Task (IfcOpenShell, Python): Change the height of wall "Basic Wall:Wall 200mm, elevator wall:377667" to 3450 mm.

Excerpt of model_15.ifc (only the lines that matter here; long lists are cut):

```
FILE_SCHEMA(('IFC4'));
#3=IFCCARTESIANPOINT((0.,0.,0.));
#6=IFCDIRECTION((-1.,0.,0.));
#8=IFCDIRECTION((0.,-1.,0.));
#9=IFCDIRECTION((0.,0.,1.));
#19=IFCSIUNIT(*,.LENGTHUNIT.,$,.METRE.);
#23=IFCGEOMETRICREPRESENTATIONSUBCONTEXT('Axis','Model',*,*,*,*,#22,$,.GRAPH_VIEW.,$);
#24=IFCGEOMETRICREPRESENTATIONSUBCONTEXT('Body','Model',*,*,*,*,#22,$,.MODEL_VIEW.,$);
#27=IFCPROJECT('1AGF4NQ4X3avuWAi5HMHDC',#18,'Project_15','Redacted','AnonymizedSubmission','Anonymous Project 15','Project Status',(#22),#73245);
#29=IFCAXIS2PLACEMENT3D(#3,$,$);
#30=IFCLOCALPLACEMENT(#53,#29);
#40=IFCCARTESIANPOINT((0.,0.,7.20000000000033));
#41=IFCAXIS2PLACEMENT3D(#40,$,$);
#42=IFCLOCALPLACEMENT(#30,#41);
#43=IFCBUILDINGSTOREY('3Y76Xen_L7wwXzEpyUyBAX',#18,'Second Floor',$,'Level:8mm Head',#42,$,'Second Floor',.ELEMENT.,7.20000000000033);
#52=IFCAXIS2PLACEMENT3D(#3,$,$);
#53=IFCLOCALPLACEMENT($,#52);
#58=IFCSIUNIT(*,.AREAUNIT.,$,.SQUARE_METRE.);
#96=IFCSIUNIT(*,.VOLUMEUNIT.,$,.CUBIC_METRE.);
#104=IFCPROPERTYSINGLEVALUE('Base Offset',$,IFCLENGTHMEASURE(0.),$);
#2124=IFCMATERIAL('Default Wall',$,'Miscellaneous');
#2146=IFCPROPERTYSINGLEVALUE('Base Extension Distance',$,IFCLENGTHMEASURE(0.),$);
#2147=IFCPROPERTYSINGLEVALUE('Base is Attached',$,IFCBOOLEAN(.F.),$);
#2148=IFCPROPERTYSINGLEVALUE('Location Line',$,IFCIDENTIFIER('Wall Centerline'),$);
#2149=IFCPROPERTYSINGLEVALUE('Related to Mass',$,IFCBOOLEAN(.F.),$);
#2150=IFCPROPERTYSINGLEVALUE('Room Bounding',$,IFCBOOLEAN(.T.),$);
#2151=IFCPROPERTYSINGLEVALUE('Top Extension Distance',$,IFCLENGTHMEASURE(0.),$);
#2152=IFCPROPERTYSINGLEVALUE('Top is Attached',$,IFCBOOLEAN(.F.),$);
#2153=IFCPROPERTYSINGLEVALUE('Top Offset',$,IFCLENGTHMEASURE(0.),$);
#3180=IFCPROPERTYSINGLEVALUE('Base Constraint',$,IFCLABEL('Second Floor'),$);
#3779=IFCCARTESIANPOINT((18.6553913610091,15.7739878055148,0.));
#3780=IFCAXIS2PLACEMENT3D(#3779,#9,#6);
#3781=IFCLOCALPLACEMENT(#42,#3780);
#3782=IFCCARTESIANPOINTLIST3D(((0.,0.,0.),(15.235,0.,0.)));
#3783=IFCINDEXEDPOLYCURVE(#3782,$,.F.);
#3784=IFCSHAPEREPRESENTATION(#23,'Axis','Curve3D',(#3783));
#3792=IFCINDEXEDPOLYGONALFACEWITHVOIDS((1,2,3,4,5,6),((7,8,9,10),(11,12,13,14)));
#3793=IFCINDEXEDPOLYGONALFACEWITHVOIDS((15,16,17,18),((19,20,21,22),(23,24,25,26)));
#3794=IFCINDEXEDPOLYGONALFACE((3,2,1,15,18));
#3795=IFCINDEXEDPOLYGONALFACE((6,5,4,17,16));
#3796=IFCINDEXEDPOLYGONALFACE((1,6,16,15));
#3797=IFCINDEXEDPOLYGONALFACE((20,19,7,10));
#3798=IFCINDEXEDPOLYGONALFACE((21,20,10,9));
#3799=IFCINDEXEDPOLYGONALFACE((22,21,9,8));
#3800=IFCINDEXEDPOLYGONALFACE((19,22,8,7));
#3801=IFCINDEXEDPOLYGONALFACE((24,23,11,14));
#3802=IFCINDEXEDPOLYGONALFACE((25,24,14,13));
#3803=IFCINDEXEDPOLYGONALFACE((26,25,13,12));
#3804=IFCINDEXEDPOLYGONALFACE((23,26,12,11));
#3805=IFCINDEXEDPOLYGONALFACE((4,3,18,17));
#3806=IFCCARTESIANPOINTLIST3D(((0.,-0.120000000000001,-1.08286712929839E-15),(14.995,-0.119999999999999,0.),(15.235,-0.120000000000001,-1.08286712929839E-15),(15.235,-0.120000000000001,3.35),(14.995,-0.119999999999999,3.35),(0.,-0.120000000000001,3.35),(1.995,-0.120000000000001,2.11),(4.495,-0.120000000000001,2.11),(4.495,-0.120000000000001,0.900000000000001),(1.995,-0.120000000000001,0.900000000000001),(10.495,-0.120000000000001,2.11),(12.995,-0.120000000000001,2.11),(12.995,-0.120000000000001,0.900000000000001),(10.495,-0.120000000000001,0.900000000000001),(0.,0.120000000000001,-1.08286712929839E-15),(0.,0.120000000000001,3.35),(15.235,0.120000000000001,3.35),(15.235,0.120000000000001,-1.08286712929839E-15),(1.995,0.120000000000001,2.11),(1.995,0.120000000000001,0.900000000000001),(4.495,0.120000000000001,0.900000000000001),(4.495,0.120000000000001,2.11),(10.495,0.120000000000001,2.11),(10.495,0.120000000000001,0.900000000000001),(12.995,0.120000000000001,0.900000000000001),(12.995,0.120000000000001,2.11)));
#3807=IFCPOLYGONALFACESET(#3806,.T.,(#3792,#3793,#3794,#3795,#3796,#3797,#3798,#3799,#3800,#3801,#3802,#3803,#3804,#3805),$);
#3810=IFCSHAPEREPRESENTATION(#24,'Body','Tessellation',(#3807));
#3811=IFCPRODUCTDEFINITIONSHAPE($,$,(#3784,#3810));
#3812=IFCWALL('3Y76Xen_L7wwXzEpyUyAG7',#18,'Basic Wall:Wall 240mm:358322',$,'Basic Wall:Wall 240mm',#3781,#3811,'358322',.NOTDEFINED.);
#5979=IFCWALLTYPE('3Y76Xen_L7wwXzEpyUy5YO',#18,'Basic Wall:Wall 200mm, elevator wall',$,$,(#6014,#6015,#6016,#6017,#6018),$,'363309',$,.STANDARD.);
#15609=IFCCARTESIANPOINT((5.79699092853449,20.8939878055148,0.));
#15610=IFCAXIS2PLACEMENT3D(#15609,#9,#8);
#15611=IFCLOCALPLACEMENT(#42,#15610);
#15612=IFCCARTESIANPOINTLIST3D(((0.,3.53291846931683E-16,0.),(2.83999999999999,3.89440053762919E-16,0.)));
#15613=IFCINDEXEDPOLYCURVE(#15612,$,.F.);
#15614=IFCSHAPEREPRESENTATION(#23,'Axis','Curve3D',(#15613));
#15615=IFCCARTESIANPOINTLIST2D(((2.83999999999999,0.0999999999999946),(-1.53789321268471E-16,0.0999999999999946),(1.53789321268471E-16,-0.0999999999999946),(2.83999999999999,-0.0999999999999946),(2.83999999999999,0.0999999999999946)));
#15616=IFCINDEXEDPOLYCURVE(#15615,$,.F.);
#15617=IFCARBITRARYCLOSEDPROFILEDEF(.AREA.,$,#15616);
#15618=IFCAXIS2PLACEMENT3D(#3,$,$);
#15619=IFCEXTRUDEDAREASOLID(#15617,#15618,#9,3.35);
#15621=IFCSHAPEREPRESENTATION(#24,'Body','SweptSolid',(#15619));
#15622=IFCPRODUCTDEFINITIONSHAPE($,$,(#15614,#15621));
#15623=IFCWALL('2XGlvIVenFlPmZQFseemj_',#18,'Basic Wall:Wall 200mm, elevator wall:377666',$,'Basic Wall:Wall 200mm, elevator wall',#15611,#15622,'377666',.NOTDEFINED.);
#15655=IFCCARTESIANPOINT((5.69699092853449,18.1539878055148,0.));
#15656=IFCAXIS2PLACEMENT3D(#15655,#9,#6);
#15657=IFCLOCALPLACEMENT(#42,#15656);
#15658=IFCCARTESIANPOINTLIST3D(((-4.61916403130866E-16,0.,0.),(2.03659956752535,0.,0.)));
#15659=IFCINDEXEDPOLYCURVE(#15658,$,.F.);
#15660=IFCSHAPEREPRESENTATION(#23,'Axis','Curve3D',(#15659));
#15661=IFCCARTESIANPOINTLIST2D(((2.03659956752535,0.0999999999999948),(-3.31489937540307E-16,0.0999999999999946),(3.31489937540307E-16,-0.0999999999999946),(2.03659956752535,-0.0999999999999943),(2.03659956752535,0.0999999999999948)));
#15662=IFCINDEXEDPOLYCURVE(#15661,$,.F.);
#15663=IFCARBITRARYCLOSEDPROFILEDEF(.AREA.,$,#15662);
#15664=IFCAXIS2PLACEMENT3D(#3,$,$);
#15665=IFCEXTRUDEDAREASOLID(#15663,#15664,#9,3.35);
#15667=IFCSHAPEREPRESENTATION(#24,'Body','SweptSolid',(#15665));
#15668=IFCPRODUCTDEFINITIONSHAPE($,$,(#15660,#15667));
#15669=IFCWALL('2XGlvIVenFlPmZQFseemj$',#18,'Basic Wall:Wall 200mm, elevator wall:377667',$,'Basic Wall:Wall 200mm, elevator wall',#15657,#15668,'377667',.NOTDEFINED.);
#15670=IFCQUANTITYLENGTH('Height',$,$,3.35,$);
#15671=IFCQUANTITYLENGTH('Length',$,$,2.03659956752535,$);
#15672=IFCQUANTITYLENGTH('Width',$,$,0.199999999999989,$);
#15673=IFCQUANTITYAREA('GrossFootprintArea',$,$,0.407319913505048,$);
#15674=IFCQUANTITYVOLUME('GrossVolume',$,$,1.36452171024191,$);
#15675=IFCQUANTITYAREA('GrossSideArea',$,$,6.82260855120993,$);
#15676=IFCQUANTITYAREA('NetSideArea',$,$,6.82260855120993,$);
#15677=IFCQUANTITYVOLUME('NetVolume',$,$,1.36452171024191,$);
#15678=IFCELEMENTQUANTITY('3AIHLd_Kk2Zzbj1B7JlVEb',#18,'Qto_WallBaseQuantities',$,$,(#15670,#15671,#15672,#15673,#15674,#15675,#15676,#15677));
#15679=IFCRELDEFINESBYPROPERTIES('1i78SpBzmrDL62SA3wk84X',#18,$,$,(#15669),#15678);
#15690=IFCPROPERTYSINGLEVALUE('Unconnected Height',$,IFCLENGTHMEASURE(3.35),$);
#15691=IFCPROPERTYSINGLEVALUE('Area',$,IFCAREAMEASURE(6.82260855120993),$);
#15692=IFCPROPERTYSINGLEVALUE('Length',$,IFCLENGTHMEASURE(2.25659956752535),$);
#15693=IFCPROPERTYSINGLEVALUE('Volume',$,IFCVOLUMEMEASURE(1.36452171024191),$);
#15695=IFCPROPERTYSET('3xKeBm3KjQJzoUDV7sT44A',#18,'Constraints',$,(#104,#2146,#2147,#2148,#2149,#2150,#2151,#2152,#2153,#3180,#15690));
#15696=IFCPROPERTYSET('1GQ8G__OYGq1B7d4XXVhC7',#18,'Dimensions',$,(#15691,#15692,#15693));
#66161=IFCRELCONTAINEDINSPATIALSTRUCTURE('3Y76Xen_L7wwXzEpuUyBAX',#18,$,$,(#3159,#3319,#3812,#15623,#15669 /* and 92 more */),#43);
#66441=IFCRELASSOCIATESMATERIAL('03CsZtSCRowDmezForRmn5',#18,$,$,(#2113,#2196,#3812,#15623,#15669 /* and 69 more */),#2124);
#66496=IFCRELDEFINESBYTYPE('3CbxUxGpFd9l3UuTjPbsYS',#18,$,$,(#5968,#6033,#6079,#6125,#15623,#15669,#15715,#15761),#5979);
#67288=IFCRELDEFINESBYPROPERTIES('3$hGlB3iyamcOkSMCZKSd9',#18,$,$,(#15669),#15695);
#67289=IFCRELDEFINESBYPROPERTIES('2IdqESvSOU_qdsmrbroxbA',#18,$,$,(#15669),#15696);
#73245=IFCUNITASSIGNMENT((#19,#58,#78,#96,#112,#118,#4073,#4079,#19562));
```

```python
import ifcopenshell
import ifcopenshell.api.pset
import ifcopenshell.geom
import ifcopenshell.util.element
import ifcopenshell.util.representation
import ifcopenshell.util.shape
import ifcopenshell.util.unit

model = ifcopenshell.open("model_15.ifc")
unit_scale = ifcopenshell.util.unit.calculate_unit_scale(model)
area_scale = ifcopenshell.util.unit.calculate_unit_scale(model, "AREAUNIT")
volume_scale = ifcopenshell.util.unit.calculate_unit_scale(model, "VOLUMEUNIT")
settings = ifcopenshell.geom.settings()


def volume(element):
    """Net volume in cubic metres, openings subtracted."""
    shape = ifcopenshell.geom.create_shape(settings, element)
    return ifcopenshell.util.shape.get_volume(shape.geometry)


wall = model.by_id(15669)
before = volume(wall)

body = ifcopenshell.util.representation.get_representation(wall, "Model", "Body")
solid = body.Items[0]
old_height = solid.Depth
solid.Depth = 3.45 / unit_scale
after = volume(wall)
thickness = 0.2  # wall thickness in metres

# Update the stored height, areas and volumes.
qto = model.by_id(ifcopenshell.util.element.get_pset(wall, "Qto_WallBaseQuantities", should_inherit=False)["id"])
ifcopenshell.api.pset.edit_qto(model, qto=qto, properties={
    "Height": solid.Depth,
    "GrossVolume": ifcopenshell.util.element.get_pset(wall, "Qto_WallBaseQuantities", "GrossVolume") * solid.Depth / old_height,
    "GrossSideArea": ifcopenshell.util.element.get_pset(wall, "Qto_WallBaseQuantities", "GrossSideArea") * solid.Depth / old_height,
    "NetSideArea": after / thickness / area_scale,
    "NetVolume": after / volume_scale,
})
pset = model.by_id(ifcopenshell.util.element.get_pset(wall, "Constraints", should_inherit=False)["id"])
ifcopenshell.api.pset.edit_pset(model, pset=pset, properties={
    "Unconnected Height": model.create_entity("IfcLengthMeasure", solid.Depth),
})
pset = model.by_id(ifcopenshell.util.element.get_pset(wall, "Dimensions", should_inherit=False)["id"])
ifcopenshell.api.pset.edit_pset(model, pset=pset, properties={
    "Area": model.create_entity("IfcAreaMeasure", after / thickness / area_scale),
    "Volume": model.create_entity("IfcVolumeMeasure", after / volume_scale),
})

print(f"height {old_height:g} -> {solid.Depth:g}, volume {before:.3f} -> {after:.3f} m3")

model.write("model_15_updated.ifc")
```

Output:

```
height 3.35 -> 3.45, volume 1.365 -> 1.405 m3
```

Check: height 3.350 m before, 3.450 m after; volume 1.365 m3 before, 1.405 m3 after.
